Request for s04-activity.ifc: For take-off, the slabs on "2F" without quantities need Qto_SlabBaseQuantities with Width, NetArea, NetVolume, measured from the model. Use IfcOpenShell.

First a look at what the model holds.

```python
import ifcopenshell
import ifcopenshell.util.element
import ifcopenshell.util.unit

model = ifcopenshell.open("s04-activity.ifc")
print(model.schema)
for unit_type in ("LENGTHUNIT", "AREAUNIT", "VOLUMEUNIT"):
    print(unit_type, ifcopenshell.util.unit.calculate_unit_scale(model, unit_type))
storey = next(s for s in model.by_type("IfcBuildingStorey") if s.Name == "2F")
slabs = [e for e in ifcopenshell.util.element.get_decomposition(storey) if e.is_a("IfcSlab")]
for e in sorted(slabs, key=lambda e: e.id()):
    print(e.id(), e.is_a(), e.Name, list(ifcopenshell.util.element.get_psets(e, qtos_only=True)), sep=" | ")
```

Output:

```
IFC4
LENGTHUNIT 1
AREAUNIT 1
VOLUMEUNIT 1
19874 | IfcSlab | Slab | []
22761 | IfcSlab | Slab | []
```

```python
import ifcopenshell
import ifcopenshell.api.pset
import ifcopenshell.geom
import ifcopenshell.util.element
import ifcopenshell.util.shape
import ifcopenshell.util.unit

model = ifcopenshell.open("s04-activity.ifc")
unit_scale = ifcopenshell.util.unit.calculate_unit_scale(model)
area_scale = ifcopenshell.util.unit.calculate_unit_scale(model, "AREAUNIT")
volume_scale = ifcopenshell.util.unit.calculate_unit_scale(model, "VOLUMEUNIT")
settings = ifcopenshell.geom.settings()

storey = next(s for s in model.by_type("IfcBuildingStorey") if s.Name == "2F")
slabs = [e for e in ifcopenshell.util.element.get_decomposition(storey) if e.is_a("IfcSlab")]

for e in sorted(slabs, key=lambda e: e.id()):
    if ifcopenshell.util.element.get_psets(e, qtos_only=True, should_inherit=False):
        continue
    # Geometry comes back in metres, in the element's own axes.
    shape = ifcopenshell.geom.create_shape(settings, e)
    values = {
        "Width": ifcopenshell.util.shape.get_z(shape.geometry) / unit_scale,
        "NetArea": ifcopenshell.util.shape.get_footprint_area(shape.geometry) / area_scale,
        "NetVolume": ifcopenshell.util.shape.get_volume(shape.geometry) / volume_scale,
    }
    qto = ifcopenshell.api.pset.add_qto(model, product=e, name="Qto_SlabBaseQuantities")
    ifcopenshell.api.pset.edit_qto(model, qto=qto, properties=values)
    print(e.id(), {k: round(v, 3) for k, v in values.items()})

model.write("s04-activity_edited.ifc")
```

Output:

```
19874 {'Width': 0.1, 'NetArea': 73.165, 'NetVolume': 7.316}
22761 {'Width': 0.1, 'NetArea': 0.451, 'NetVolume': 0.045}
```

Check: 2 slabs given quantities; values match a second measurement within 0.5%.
